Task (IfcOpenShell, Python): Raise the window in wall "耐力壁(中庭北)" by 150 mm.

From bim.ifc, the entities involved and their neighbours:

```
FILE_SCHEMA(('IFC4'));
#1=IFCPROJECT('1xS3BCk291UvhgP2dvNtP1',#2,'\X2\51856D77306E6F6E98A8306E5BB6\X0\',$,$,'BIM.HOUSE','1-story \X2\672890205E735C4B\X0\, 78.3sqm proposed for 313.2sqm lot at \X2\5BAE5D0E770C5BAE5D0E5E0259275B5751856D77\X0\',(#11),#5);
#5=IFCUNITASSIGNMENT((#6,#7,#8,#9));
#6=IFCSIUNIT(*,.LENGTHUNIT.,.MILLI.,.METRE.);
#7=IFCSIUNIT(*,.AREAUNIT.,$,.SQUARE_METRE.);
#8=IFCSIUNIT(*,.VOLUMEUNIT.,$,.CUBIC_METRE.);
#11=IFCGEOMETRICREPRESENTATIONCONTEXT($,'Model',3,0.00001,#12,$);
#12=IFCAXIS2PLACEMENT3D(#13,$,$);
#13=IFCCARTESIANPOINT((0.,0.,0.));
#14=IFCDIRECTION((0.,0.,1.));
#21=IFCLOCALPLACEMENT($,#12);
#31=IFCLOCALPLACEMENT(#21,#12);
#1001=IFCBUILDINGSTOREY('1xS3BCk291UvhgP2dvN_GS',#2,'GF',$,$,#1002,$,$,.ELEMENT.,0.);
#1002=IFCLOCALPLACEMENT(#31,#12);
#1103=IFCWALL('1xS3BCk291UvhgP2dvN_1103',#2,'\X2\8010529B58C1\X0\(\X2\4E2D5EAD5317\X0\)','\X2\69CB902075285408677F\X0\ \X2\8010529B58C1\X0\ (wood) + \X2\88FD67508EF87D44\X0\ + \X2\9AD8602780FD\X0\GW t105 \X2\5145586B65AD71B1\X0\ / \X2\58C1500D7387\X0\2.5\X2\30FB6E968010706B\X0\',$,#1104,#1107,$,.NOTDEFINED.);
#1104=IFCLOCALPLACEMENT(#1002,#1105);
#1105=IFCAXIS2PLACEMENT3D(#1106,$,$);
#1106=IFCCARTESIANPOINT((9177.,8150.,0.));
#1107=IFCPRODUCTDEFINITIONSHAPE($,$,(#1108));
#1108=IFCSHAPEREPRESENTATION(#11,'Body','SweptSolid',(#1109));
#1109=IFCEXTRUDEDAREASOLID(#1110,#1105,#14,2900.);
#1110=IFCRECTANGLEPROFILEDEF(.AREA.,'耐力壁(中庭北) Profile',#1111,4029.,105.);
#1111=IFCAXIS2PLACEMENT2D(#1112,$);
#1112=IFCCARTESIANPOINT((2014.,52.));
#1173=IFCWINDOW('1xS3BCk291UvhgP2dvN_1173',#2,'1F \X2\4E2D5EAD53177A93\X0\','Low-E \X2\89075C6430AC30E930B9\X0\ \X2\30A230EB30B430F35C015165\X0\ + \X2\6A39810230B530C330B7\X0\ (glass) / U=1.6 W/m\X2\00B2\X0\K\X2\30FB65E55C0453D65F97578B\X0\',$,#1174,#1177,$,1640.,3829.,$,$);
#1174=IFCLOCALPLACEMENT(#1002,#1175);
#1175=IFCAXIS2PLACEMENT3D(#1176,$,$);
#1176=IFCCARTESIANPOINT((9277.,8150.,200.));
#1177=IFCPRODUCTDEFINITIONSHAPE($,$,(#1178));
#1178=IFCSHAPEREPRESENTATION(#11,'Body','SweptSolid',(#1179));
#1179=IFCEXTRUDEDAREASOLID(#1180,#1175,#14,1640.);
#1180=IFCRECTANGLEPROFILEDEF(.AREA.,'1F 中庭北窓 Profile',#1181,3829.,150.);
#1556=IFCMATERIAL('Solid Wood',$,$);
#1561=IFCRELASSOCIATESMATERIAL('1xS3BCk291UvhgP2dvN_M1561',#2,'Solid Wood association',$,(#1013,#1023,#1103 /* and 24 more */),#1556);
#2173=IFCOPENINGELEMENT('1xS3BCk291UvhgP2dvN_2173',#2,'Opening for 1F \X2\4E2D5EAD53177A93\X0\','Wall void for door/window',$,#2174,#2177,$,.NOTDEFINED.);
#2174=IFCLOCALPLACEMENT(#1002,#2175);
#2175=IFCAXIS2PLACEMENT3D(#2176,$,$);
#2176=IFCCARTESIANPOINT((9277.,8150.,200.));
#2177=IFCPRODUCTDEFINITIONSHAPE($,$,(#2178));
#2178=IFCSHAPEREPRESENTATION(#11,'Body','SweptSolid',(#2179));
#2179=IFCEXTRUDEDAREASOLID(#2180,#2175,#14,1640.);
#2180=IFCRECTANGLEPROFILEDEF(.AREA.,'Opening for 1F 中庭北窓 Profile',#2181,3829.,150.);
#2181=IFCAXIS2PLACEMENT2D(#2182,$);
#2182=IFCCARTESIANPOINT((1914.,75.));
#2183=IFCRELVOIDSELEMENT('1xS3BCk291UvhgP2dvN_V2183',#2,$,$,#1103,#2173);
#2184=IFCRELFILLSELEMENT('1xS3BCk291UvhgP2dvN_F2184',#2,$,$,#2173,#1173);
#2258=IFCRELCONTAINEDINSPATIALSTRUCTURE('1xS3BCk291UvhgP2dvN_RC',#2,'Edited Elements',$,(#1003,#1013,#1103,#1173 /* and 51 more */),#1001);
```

```python
import numpy as np
import ifcopenshell
import ifcopenshell.api.geometry
import ifcopenshell.util.placement
import ifcopenshell.util.unit

model = ifcopenshell.open("bim.ifc")
unit_scale = ifcopenshell.util.unit.calculate_unit_scale(model)

window = model.by_id(1173)
opening = window.FillsVoids[0].RelatingOpeningElement
dz = 0.15 / unit_scale

shift = np.array([0.0, 0.0, dz])
# The window is not placed relative to its opening, so move both.
for product in (opening, window):
    matrix = ifcopenshell.util.placement.get_local_placement(product.ObjectPlacement)
    matrix[:3, 3] += shift
    ifcopenshell.api.geometry.edit_object_placement(model, product=product, matrix=matrix, is_si=False)

print(f"moved by {dz * unit_scale:+.3f} m")

model.write("bim_rev.ifc")
```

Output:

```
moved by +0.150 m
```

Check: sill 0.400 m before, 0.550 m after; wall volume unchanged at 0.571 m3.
